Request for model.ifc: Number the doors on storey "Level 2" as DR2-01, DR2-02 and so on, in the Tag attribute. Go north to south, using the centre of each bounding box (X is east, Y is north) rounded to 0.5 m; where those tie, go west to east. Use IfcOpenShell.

First a look at what the model holds.

```python
import ifcopenshell
import ifcopenshell.util.element
import ifcopenshell.util.placement

model = ifcopenshell.open("model.ifc")
print(model.schema)
storey = next(s for s in model.by_type("IfcBuildingStorey") if s.Name == "Level 2")
doors = [e for e in ifcopenshell.util.element.get_decomposition(storey) if e.is_a("IfcDoor")]
for e in sorted(doors, key=lambda e: e.id()):
    origin = ifcopenshell.util.placement.get_local_placement(e.ObjectPlacement)[:3, 3]
    print(e.id(), e.Tag, e.Name, origin.round(2) + 0.0, sep=" | ")
```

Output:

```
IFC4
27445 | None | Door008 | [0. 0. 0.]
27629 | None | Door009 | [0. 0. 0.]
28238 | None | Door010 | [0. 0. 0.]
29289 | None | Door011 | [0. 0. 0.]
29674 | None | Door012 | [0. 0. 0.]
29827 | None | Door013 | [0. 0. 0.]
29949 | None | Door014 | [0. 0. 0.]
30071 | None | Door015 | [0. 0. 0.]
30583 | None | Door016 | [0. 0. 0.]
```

```python
import ifcopenshell
import ifcopenshell.geom
import ifcopenshell.util.element
import ifcopenshell.util.shape

model = ifcopenshell.open("model.ifc")
settings = ifcopenshell.geom.settings()
settings.set("use-world-coords", True)


def centre(element):
    shape = ifcopenshell.geom.create_shape(settings, element)
    return ifcopenshell.util.shape.get_bbox_centroid(shape.geometry)


storey = next(s for s in model.by_type("IfcBuildingStorey") if s.Name == "Level 2")
doors = [e for e in ifcopenshell.util.element.get_decomposition(storey) if e.is_a("IfcDoor")]

# Insertion points can sit at a corner or the storey origin, so sort by the geometry (in metres).
centres = {e: centre(e) for e in doors}
doors.sort(key=lambda e: (-round(centres[e][1] / 0.5), centres[e][0]))

for i, e in enumerate(doors, start=1):
    number = f"DR2-{i:02d}"
    e.Tag = number
    print(e.id(), number)

model.write("model_v2.ifc")
```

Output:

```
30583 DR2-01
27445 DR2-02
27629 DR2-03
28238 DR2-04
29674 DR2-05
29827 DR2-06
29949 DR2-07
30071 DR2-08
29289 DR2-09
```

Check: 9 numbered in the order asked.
